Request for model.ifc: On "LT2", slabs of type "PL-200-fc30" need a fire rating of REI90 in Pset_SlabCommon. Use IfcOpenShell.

First a look at what the model holds.

```python
import ifcopenshell
import ifcopenshell.util.element

model = ifcopenshell.open("model.ifc")
print(model.schema)
storey = next(s for s in model.by_type("IfcBuildingStorey") if s.Name == "LT2")
slabs = [e for e in ifcopenshell.util.element.get_decomposition(storey) if e.is_a("IfcSlab")]
seen = {}
for e in slabs:
    element_type = ifcopenshell.util.element.get_type(e)
    key = (element_type.Name if element_type != e and element_type else None, ifcopenshell.util.element.get_pset(e, "Pset_SlabCommon", "FireRating"))
    seen[key] = seen.get(key, 0) + 1
for (name, value), count in sorted(seen.items(), key=str):
    print(count, "x", name, "|", value)
```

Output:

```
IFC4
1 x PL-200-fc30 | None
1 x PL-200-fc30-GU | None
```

```python
import ifcopenshell
import ifcopenshell.api.pset
import ifcopenshell.util.element

model = ifcopenshell.open("model.ifc")

storey = next(s for s in model.by_type("IfcBuildingStorey") if s.Name == "LT2")
slabs = [e for e in ifcopenshell.util.element.get_decomposition(storey) if e.is_a("IfcSlab")]

count = 0
for e in slabs:
    element_type = ifcopenshell.util.element.get_type(e)
    if element_type in (None, e) or element_type.Name != "PL-200-fc30":
        continue
    # add_pset returns the element's existing set when there is one.
    pset = ifcopenshell.api.pset.add_pset(model, product=e, name="Pset_SlabCommon")
    ifcopenshell.api.pset.edit_pset(model, pset=pset, properties={"FireRating": "REI90"})
    count += 1

print(count, "slabs updated")

model.write("model_edited.ifc")
```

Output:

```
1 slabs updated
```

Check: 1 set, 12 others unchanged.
